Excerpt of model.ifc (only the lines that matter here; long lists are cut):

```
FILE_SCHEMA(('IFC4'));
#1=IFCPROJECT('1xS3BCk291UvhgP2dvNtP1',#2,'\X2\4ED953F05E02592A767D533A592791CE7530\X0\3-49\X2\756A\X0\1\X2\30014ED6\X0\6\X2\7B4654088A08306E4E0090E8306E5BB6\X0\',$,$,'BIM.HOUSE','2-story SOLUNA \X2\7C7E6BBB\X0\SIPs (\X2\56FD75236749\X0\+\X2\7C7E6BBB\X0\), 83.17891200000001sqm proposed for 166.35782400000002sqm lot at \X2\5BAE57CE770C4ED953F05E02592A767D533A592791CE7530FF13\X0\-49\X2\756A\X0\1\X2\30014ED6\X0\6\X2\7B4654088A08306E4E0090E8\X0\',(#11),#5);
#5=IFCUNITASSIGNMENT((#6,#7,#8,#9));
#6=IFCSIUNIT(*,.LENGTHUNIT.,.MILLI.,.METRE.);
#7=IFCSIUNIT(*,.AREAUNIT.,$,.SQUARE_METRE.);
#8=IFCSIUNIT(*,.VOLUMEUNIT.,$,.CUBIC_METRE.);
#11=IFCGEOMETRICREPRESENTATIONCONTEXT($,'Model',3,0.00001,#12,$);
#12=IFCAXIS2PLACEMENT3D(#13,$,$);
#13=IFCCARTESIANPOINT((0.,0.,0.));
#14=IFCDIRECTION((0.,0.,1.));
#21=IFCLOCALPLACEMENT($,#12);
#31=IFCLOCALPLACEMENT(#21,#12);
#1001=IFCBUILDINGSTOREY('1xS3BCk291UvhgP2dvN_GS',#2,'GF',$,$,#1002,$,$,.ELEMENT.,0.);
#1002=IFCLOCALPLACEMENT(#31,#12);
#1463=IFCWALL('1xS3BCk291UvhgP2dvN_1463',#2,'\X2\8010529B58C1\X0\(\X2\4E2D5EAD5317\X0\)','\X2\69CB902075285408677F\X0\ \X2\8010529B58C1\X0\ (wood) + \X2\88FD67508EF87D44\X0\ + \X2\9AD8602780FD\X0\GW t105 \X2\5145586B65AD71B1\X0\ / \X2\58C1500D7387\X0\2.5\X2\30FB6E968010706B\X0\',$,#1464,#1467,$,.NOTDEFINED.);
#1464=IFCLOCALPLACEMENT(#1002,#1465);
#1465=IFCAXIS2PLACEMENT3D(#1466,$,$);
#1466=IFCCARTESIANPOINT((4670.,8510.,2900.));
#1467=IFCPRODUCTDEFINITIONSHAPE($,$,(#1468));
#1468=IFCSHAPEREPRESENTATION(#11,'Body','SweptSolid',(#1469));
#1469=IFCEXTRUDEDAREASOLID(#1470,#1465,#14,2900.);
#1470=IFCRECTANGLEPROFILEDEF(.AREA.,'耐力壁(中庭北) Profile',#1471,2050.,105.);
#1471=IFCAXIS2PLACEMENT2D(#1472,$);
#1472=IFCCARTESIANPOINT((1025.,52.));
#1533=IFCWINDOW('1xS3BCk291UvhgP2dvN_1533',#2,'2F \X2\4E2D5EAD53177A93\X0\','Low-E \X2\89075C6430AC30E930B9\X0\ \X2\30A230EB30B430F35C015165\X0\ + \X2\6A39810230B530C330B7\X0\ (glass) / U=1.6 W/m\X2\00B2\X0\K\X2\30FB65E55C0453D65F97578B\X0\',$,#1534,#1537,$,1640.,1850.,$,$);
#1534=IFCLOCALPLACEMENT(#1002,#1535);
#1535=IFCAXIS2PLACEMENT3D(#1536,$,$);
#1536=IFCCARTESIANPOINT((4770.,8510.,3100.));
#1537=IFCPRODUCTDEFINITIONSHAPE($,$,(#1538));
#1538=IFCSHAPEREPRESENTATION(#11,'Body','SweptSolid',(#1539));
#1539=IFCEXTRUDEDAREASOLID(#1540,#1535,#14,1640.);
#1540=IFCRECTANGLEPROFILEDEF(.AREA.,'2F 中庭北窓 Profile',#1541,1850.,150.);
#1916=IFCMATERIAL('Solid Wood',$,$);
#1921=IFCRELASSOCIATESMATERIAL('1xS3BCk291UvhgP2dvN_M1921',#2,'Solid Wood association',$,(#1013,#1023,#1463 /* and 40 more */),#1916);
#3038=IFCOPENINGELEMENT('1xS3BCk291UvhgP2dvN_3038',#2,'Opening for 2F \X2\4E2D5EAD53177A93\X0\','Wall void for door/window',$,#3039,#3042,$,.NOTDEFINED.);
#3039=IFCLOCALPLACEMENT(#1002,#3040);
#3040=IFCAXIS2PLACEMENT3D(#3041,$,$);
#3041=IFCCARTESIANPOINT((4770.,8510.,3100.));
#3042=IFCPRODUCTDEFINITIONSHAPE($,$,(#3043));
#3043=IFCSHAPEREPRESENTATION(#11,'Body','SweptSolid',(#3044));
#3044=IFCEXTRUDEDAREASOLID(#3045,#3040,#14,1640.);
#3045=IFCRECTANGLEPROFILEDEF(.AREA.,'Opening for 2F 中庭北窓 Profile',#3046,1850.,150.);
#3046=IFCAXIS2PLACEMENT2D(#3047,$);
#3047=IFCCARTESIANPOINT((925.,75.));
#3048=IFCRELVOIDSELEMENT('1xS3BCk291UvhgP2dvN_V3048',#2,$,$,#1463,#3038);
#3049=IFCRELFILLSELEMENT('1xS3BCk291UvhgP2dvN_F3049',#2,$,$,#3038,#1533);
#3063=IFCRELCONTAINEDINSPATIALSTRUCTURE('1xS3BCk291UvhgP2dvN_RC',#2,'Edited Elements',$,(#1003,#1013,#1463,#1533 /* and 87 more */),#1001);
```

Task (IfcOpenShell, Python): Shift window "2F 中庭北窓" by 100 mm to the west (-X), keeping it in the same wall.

```python
import ifcopenshell
import ifcopenshell.api.geometry
import ifcopenshell.util.placement

model = ifcopenshell.open("model.ifc")

window = model.by_guid("1xS3BCk291UvhgP2dvN_1533")
opening = window.FillsVoids[0].RelatingOpeningElement
wall = opening.VoidsElements[0].RelatingBuildingElement

wall_matrix = ifcopenshell.util.placement.get_local_placement(wall.ObjectPlacement)
shift = wall_matrix[:3, 0] * -100.0
before = ifcopenshell.util.placement.get_local_placement(window.ObjectPlacement)[:3, 3].copy()

# The window is not placed relative to its opening, so move both.
for product in (opening, window):
    matrix = ifcopenshell.util.placement.get_local_placement(product.ObjectPlacement)
    matrix[:3, 3] += shift
    ifcopenshell.api.geometry.edit_object_placement(model, product=product, matrix=matrix, is_si=False)

after = ifcopenshell.util.placement.get_local_placement(window.ObjectPlacement)[:3, 3]
print("window moved by", (after - before).round(3) + 0.0)

model.write("model_v2.ifc")
```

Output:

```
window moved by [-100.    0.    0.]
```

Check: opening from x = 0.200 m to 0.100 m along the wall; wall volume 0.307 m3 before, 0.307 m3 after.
